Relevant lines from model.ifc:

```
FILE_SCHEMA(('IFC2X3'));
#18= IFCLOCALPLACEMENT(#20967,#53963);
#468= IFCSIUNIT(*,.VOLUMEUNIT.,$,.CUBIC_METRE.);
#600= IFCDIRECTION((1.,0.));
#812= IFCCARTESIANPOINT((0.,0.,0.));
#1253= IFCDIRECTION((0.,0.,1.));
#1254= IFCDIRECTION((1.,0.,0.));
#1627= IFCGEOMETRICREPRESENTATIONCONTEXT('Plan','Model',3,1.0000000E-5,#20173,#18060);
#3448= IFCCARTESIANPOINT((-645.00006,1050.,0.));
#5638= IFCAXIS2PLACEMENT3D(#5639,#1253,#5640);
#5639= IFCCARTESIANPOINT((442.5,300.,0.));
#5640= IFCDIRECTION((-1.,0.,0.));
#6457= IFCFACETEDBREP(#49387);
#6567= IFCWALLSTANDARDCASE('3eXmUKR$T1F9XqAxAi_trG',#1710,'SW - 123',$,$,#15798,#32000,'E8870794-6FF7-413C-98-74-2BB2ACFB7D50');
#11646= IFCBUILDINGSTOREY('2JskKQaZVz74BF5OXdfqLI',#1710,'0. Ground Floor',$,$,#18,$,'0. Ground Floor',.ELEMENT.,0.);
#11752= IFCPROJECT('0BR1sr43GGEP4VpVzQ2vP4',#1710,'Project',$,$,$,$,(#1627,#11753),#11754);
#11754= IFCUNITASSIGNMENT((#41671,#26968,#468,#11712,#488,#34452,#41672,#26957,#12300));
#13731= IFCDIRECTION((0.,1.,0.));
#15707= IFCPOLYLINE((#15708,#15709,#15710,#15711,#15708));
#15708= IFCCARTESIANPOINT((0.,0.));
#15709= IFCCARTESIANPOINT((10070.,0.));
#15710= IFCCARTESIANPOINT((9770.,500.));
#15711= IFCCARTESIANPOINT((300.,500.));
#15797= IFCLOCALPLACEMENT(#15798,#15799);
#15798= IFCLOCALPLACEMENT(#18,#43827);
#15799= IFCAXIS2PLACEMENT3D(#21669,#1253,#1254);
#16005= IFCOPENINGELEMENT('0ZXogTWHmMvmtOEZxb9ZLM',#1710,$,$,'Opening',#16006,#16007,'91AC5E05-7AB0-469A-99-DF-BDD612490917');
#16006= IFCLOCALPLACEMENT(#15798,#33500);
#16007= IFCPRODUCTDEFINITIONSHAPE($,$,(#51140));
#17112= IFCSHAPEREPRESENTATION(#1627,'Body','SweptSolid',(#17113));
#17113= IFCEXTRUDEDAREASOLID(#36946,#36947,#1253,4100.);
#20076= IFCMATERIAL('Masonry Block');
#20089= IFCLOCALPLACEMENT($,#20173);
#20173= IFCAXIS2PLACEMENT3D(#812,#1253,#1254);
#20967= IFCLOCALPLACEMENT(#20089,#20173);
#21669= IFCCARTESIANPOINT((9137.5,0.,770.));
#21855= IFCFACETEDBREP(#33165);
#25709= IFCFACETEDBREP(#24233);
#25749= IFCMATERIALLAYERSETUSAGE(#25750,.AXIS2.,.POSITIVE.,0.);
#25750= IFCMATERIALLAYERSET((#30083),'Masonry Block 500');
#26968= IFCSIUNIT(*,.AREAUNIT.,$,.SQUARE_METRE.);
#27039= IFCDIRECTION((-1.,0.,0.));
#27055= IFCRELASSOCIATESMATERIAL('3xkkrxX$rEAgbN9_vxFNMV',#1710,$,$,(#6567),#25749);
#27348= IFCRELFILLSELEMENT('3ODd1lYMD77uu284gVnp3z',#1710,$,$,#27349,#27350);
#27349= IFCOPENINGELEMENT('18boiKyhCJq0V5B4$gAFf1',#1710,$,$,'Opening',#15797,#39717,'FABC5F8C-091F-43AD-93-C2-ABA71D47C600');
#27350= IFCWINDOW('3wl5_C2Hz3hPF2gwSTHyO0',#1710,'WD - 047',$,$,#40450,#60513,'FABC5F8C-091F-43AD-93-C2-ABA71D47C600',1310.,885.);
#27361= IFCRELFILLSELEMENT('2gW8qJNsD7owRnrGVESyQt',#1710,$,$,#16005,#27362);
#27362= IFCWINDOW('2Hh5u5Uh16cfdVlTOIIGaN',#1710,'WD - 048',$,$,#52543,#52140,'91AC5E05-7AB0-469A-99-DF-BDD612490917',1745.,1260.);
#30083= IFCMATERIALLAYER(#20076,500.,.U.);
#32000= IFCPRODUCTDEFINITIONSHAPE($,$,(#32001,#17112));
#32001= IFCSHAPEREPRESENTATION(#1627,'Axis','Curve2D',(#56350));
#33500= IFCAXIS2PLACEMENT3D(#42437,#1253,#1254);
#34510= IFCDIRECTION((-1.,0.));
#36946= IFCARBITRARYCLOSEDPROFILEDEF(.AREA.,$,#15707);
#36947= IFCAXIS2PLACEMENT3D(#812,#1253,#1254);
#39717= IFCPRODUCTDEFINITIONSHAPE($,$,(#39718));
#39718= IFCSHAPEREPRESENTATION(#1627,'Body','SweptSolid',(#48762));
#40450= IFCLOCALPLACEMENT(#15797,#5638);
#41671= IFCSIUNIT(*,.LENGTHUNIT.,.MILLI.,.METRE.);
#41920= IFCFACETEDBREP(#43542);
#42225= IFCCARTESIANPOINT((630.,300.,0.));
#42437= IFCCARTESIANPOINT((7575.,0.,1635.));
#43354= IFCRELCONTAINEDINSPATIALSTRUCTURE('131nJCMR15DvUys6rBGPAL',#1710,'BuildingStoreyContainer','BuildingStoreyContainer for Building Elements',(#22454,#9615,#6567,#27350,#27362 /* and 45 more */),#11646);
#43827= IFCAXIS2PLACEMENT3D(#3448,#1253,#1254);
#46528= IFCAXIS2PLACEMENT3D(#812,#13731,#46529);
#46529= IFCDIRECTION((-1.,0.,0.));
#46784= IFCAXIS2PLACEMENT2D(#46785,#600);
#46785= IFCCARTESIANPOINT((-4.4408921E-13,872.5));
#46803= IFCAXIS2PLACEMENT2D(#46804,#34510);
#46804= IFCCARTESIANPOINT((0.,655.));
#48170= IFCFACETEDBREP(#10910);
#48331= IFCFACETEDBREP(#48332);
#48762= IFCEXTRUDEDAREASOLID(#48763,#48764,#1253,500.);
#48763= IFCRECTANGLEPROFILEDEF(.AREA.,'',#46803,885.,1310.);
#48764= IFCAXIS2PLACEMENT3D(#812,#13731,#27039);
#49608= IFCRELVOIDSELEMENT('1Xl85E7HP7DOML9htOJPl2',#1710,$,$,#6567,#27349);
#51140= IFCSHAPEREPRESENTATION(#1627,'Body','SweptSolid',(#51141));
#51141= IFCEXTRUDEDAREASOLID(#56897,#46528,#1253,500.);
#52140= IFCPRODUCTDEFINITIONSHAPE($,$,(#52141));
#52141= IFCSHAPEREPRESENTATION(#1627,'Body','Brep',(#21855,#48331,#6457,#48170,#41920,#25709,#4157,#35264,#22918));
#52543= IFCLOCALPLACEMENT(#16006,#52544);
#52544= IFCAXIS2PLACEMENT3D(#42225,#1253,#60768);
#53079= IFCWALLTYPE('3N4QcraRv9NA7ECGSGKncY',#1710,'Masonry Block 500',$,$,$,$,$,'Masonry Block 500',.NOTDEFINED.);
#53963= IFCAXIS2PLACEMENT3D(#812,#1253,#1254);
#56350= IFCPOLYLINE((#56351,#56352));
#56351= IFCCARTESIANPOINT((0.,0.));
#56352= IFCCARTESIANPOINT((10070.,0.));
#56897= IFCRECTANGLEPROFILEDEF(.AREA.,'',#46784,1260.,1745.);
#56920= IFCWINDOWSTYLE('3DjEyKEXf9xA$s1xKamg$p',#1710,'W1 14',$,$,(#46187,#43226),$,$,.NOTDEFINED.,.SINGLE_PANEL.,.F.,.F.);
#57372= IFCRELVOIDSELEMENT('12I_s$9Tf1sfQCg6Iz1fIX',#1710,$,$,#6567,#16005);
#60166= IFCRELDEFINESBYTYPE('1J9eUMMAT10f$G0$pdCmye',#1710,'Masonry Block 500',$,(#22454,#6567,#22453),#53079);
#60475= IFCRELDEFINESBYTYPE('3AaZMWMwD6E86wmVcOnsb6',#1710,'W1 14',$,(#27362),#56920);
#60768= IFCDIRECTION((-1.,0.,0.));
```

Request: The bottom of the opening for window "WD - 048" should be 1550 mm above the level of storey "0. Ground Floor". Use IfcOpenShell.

```python
import numpy as np
import ifcopenshell
import ifcopenshell.api.geometry
import ifcopenshell.geom
import ifcopenshell.util.element
import ifcopenshell.util.placement
import ifcopenshell.util.shape
import ifcopenshell.util.unit

model = ifcopenshell.open("model.ifc")
unit_scale = ifcopenshell.util.unit.calculate_unit_scale(model)

window = model.by_guid("2Hh5u5Uh16cfdVlTOIIGaN")
opening = window.FillsVoids[0].RelatingOpeningElement
storey = ifcopenshell.util.element.get_container(window, ifc_class="IfcBuildingStorey")
level = ifcopenshell.util.placement.get_local_placement(storey.ObjectPlacement)[2, 3]

# The opening's origin need not be at the sill, so measure its lowest point.
shape = ifcopenshell.geom.create_shape(ifcopenshell.geom.settings(), opening)
bottom = ifcopenshell.util.shape.get_shape_bottom_elevation(shape, shape.geometry) / unit_scale
dz = level + 1550.0 - bottom

shift = np.array([0.0, 0.0, dz])
# The window is placed relative to its opening, so it follows when the opening moves.
matrix = ifcopenshell.util.placement.get_local_placement(opening.ObjectPlacement)
matrix[:3, 3] += shift
ifcopenshell.api.geometry.edit_object_placement(
    model, product=opening, matrix=matrix, is_si=False, should_transform_children=True
)

print(f"moved by {dz * unit_scale:+.3f} m")

model.write("model_v2.ifc")
```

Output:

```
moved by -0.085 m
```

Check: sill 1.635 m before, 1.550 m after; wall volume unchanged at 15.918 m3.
